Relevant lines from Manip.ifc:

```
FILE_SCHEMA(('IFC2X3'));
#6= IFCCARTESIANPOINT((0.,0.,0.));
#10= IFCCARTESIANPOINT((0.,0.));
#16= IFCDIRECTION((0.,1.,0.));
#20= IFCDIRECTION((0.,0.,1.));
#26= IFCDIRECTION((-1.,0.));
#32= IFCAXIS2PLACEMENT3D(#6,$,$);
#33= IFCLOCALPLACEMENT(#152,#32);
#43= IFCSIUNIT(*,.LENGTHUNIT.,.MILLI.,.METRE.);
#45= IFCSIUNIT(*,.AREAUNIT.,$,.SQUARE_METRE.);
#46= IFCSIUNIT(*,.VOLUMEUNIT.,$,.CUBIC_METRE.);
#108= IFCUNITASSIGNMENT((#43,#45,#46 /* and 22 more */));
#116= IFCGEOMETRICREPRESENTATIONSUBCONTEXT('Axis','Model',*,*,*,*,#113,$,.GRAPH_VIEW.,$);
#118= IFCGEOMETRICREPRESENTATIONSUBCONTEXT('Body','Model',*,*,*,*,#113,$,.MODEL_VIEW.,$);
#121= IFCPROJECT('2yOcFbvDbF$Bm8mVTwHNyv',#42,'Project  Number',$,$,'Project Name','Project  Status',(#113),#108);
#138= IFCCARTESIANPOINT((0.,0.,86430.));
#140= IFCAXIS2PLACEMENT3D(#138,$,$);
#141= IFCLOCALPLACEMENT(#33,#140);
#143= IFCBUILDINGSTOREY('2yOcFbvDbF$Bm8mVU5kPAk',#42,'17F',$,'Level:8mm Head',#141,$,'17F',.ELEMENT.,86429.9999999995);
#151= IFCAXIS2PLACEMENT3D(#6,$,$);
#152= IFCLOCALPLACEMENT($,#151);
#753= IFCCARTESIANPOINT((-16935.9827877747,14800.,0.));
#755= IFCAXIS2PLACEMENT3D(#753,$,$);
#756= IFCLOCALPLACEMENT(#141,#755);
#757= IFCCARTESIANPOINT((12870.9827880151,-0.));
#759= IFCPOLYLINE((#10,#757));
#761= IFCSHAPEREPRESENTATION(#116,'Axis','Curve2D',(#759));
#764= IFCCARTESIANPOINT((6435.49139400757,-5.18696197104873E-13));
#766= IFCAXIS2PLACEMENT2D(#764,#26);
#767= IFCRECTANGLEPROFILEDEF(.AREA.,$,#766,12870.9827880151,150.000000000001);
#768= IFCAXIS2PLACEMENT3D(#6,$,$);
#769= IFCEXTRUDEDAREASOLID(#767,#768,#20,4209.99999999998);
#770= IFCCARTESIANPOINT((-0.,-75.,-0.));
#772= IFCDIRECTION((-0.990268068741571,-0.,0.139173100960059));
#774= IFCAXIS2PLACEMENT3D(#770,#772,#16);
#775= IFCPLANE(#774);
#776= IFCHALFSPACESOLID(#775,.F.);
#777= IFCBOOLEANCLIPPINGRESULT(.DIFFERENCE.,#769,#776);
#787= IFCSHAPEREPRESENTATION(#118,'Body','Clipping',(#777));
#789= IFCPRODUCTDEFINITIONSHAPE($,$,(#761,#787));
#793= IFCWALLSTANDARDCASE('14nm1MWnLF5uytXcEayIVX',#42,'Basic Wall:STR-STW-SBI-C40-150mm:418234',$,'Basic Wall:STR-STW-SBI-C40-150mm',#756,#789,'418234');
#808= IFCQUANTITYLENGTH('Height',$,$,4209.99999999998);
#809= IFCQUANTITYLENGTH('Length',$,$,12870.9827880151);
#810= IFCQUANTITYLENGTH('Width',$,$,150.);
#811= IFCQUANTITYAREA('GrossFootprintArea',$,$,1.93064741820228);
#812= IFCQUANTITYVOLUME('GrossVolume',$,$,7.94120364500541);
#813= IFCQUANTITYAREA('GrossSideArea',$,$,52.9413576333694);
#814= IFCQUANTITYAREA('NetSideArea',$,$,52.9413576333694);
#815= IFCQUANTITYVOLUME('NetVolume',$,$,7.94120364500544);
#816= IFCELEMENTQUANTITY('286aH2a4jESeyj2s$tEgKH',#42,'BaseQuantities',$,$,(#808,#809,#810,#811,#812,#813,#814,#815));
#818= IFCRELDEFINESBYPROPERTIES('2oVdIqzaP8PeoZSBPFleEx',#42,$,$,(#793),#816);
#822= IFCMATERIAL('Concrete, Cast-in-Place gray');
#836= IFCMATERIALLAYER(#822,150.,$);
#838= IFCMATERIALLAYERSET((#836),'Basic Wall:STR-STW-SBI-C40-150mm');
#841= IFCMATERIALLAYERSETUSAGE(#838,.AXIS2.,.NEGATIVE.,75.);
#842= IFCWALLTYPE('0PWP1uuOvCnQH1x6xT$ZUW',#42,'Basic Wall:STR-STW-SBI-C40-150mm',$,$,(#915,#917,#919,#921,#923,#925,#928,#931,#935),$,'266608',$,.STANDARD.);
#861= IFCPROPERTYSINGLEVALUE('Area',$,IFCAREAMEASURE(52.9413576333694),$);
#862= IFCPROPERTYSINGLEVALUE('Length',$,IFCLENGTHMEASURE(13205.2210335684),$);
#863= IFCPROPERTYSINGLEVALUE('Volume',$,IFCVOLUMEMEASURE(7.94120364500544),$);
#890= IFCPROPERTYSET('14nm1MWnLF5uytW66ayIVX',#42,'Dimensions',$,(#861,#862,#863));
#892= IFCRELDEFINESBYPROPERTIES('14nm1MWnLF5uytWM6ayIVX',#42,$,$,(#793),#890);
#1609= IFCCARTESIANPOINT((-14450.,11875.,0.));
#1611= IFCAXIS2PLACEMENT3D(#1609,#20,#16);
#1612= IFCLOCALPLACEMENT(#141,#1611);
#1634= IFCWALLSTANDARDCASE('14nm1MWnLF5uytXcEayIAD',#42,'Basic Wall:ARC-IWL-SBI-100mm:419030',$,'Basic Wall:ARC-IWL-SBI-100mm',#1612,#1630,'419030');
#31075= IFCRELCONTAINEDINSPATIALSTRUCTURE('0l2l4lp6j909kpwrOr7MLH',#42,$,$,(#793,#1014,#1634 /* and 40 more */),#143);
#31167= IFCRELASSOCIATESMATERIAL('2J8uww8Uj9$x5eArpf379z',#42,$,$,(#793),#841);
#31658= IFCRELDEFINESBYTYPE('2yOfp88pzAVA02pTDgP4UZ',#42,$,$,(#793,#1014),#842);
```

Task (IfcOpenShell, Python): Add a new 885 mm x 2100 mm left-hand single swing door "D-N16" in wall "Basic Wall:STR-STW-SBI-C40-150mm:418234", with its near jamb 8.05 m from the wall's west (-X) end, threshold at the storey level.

```python
import numpy as np
import ifcopenshell
import ifcopenshell.api.feature
import ifcopenshell.api.geometry
import ifcopenshell.api.pset
import ifcopenshell.api.root
import ifcopenshell.api.spatial
import ifcopenshell.api.type
import ifcopenshell.geom
import ifcopenshell.util.element
import ifcopenshell.util.placement
import ifcopenshell.util.representation
import ifcopenshell.util.shape
import ifcopenshell.util.unit

model = ifcopenshell.open("Manip.ifc")
unit_scale = ifcopenshell.util.unit.calculate_unit_scale(model)
area_scale = ifcopenshell.util.unit.calculate_unit_scale(model, "AREAUNIT")
volume_scale = ifcopenshell.util.unit.calculate_unit_scale(model, "VOLUMEUNIT")
settings = ifcopenshell.geom.settings()


def volume(element):
    """Net volume in cubic metres, openings subtracted."""
    shape = ifcopenshell.geom.create_shape(settings, element)
    return ifcopenshell.util.shape.get_volume(shape.geometry)


wall = model.by_guid("14nm1MWnLF5uytXcEayIVX")
storey = ifcopenshell.util.element.get_container(wall, ifc_class="IfcBuildingStorey")
context = ifcopenshell.util.representation.get_context(model, "Model", "Body", "MODEL_VIEW")
before = volume(wall)

width, height, from_end, sill = 0.885, 2.1, 8.05, 0.0  # metres

# The wall runs along its own X axis, and the end named is its -X end.
wall_shape = ifcopenshell.geom.create_shape(settings, wall)
x, y, z = ifcopenshell.util.shape.get_vertices(wall_shape.geometry).T
start = x.min() + from_end
face, thickness = float(y.min()), float(y.max() - y.min())
wall_matrix = ifcopenshell.util.placement.get_local_placement(wall.ObjectPlacement)
level = ifcopenshell.util.placement.get_local_placement(storey.ObjectPlacement)[2, 3]


def in_wall(x, y):
    """Placement at x, y metres in the wall's axes, at sill height."""
    matrix = wall_matrix.copy()
    matrix[:, 3] = wall_matrix @ np.array([x / unit_scale, y / unit_scale, 0.0, 1.0])
    matrix[2, 3] = level + sill / unit_scale
    return matrix


# Opening: a box that overshoots both wall faces by 50 mm.
opening = ifcopenshell.api.root.create_entity(model, ifc_class="IfcOpeningElement")
box = ifcopenshell.api.geometry.add_wall_representation(
    model, context=context, length=width, height=height, thickness=thickness + 0.1
)
ifcopenshell.api.geometry.assign_representation(model, product=opening, representation=box)
ifcopenshell.api.geometry.edit_object_placement(model, product=opening, matrix=in_wall(start, face - 0.05), is_si=False)
ifcopenshell.api.feature.add_feature(model, feature=opening, element=wall)

door = ifcopenshell.api.root.create_entity(model, ifc_class="IfcDoor", name="D-N16")
door.OverallWidth, door.OverallHeight = width / unit_scale, height / unit_scale
body = ifcopenshell.api.geometry.add_door_representation(
    model,
    context=context,
    overall_width=door.OverallWidth,
    overall_height=door.OverallHeight,
    operation_type="SINGLE_SWING_LEFT",
    lining_properties={"LiningDepth": thickness / unit_scale, "ThresholdDepth": thickness / unit_scale},
)
ifcopenshell.api.geometry.assign_representation(model, product=door, representation=body)
ifcopenshell.api.spatial.assign_container(model, products=[door], relating_structure=storey)
fills = ifcopenshell.api.feature.add_filling(model, opening=opening, element=door)
fills.OwnerHistory = door.OwnerHistory  # required in IFC2X3

# IFC2X3 keeps the operation on the door style.
style = ifcopenshell.api.root.create_entity(model, ifc_class="IfcDoorStyle", name="D-N16")
style.OperationType, style.ConstructionType = "SINGLE_SWING_LEFT", "NOTDEFINED"
style.ParameterTakesPrecedence = style.Sizeable = False
ifcopenshell.api.type.assign_type(model, related_objects=[door], relating_type=style)

# The lining spans the wall, so the door starts at the wall face.
ifcopenshell.api.geometry.edit_object_placement(model, product=door, matrix=in_wall(start, face), is_si=False)

after = volume(wall)

# Update the wall's stored quantities.
qto = model.by_id(ifcopenshell.util.element.get_pset(wall, "BaseQuantities", should_inherit=False)["id"])
ifcopenshell.api.pset.edit_qto(model, qto=qto, properties={
    "NetSideArea": after / thickness / area_scale,
    "NetVolume": after / volume_scale,
})
pset = model.by_id(ifcopenshell.util.element.get_pset(wall, "Dimensions", should_inherit=False)["id"])
ifcopenshell.api.pset.edit_pset(model, pset=pset, properties={
    "Area": model.create_entity("IfcAreaMeasure", after / thickness / area_scale),
    "Volume": model.create_entity("IfcVolumeMeasure", after / volume_scale),
})

print(f"wall volume {before:.3f} -> {after:.3f} m3")

model.write("Manip_updated.ifc")
```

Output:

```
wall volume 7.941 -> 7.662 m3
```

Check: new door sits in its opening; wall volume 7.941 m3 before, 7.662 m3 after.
